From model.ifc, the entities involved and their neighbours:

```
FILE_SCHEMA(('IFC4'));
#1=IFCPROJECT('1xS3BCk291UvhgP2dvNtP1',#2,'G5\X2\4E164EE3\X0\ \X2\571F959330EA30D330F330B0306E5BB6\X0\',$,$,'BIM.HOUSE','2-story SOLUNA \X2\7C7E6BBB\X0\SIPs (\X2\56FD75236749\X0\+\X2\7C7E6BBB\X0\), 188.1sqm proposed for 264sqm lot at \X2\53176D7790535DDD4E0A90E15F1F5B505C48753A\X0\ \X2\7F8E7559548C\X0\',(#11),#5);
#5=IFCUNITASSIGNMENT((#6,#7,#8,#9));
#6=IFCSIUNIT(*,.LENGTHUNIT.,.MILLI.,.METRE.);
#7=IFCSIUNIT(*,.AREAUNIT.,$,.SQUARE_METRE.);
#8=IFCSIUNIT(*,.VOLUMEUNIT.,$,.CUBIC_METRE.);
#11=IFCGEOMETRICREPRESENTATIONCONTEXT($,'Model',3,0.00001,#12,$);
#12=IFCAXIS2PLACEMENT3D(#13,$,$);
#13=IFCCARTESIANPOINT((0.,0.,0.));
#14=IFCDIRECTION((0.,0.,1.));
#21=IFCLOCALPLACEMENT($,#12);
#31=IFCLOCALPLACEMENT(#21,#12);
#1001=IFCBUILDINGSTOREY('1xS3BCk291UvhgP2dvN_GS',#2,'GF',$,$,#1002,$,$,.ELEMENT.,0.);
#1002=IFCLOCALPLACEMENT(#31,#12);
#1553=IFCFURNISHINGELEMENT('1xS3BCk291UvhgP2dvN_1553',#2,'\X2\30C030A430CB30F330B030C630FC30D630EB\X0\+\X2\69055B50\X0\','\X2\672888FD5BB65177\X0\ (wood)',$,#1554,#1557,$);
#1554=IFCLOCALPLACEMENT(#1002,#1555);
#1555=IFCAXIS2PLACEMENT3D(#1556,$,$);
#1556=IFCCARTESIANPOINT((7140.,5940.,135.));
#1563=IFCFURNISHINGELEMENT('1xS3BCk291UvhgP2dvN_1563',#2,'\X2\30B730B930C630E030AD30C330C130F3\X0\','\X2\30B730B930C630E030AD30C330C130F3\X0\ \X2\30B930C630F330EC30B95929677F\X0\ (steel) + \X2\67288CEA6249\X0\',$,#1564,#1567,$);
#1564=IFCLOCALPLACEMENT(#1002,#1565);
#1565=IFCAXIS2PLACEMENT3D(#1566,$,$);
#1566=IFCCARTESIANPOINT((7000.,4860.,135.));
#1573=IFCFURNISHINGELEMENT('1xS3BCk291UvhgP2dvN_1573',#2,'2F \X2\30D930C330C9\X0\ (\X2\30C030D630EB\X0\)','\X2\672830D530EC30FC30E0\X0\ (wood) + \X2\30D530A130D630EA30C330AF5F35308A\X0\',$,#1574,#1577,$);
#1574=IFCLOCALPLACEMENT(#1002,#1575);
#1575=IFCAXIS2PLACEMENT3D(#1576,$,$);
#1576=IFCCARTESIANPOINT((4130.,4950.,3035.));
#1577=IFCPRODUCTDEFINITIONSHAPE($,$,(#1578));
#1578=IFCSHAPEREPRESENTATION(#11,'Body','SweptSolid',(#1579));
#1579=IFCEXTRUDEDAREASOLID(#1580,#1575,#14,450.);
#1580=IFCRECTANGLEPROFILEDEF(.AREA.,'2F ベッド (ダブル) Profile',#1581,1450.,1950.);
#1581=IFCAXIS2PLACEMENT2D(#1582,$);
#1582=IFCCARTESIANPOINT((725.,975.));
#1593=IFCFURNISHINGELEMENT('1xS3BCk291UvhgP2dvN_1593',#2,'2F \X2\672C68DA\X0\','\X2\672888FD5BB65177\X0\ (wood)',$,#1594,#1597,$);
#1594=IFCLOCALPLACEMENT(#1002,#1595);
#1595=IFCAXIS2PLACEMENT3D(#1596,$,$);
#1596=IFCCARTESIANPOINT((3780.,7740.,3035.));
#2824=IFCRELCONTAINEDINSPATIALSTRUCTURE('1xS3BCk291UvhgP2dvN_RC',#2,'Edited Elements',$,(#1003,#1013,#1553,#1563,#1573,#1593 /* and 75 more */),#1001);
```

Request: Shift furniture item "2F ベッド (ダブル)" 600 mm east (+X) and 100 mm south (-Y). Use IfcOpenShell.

```python
import ifcopenshell
import ifcopenshell.api.geometry
import ifcopenshell.util.placement

model = ifcopenshell.open("model.ifc")

item = model.by_id(1573)
matrix = ifcopenshell.util.placement.get_local_placement(item.ObjectPlacement)
matrix[0, 3] += 600.0
matrix[1, 3] -= 100.0
ifcopenshell.api.geometry.edit_object_placement(model, product=item, matrix=matrix, is_si=False)

print(ifcopenshell.util.placement.get_local_placement(item.ObjectPlacement).round(3) + 0.0)

model.write("model-out.ifc")
```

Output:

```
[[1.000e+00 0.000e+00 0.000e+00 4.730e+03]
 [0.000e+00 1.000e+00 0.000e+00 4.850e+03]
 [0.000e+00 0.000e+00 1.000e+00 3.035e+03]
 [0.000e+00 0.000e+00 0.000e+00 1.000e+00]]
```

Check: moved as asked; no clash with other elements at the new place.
